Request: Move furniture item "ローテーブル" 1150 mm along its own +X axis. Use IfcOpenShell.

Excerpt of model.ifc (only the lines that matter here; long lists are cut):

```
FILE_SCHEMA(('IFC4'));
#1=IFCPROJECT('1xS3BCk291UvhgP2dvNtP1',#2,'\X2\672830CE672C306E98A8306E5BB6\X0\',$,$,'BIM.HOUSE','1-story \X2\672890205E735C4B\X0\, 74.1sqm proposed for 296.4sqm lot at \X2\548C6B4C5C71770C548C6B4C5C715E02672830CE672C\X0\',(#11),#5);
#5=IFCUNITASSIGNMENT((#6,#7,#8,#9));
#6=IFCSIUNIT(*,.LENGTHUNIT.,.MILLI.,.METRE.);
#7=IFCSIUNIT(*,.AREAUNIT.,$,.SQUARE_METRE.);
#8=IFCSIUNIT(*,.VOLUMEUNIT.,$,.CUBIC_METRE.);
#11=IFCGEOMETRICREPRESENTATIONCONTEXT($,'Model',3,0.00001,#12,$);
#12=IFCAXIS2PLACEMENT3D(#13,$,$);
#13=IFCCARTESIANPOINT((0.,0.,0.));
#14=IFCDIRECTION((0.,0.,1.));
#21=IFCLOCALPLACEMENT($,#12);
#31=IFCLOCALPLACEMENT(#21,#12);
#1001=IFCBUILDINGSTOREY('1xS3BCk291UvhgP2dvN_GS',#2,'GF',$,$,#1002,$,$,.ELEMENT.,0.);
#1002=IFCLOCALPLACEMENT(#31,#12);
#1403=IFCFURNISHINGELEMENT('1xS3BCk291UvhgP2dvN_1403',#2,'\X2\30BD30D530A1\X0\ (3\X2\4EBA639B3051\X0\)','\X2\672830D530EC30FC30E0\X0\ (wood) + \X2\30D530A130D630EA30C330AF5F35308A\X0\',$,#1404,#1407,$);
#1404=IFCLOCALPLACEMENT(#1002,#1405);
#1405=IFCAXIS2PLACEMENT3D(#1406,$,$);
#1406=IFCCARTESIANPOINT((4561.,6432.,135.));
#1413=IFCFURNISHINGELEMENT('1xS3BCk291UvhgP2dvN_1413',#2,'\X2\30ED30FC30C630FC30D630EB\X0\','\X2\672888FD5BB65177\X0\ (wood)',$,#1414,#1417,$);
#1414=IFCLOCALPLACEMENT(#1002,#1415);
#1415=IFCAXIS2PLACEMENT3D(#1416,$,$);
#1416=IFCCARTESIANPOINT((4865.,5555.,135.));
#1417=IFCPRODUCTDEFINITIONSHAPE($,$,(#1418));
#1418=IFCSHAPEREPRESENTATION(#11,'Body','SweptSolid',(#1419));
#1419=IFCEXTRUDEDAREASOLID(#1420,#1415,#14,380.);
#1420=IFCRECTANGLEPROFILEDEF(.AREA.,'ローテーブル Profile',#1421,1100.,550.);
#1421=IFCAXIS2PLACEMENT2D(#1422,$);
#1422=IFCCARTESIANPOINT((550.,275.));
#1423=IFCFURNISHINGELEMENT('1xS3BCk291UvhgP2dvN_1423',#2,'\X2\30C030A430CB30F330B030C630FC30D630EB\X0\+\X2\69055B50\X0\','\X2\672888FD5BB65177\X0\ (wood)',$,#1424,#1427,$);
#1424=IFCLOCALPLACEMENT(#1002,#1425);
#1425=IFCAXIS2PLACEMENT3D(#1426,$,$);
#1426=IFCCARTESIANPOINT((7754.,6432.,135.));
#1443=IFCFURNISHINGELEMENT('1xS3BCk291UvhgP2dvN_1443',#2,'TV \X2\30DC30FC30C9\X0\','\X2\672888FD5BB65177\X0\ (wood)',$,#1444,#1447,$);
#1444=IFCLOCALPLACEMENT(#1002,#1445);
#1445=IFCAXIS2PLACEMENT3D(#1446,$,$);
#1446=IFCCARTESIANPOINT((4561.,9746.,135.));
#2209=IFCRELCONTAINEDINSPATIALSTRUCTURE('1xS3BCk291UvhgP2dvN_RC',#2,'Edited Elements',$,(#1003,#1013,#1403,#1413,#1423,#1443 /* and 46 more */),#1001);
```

```python
import ifcopenshell
import ifcopenshell.api.geometry
import ifcopenshell.util.placement
import ifcopenshell.util.unit

model = ifcopenshell.open("model.ifc")
unit_scale = ifcopenshell.util.unit.calculate_unit_scale(model)

item = model.by_guid("1xS3BCk291UvhgP2dvN_1413")
matrix = ifcopenshell.util.placement.get_local_placement(item.ObjectPlacement)
matrix[:3, 3] += matrix[:3, 0] * 1.15 / unit_scale
ifcopenshell.api.geometry.edit_object_placement(model, product=item, matrix=matrix, is_si=False)

print(ifcopenshell.util.placement.get_local_placement(item.ObjectPlacement).round(3) + 0.0)

model.write("model_edited.ifc")
```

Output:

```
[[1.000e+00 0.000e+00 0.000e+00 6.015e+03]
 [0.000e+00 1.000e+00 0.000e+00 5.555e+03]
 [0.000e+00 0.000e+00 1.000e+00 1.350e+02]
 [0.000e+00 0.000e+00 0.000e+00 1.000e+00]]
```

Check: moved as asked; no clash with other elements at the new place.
